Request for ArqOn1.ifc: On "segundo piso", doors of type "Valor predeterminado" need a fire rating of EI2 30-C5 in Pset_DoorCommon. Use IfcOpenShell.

First a look at what the model holds.

```python
import ifcopenshell
import ifcopenshell.util.element

model = ifcopenshell.open("ArqOn1.ifc")
print(model.schema)
storey = next(s for s in model.by_type("IfcBuildingStorey") if s.Name == "segundo piso")
doors = [e for e in ifcopenshell.util.element.get_decomposition(storey) if e.is_a("IfcDoor")]
seen = {}
for e in doors:
    element_type = ifcopenshell.util.element.get_type(e)
    key = (element_type.Name if element_type != e and element_type else None, ifcopenshell.util.element.get_pset(e, "Pset_DoorCommon", "FireRating"))
    seen[key] = seen.get(key, 0) + 1
for (name, value), count in sorted(seen.items(), key=str):
    print(count, "x", name, "|", value)
```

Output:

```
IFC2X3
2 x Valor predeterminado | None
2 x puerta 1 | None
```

```python
import ifcopenshell
import ifcopenshell.api.pset
import ifcopenshell.util.element

model = ifcopenshell.open("ArqOn1.ifc")

storey = next(s for s in model.by_type("IfcBuildingStorey") if s.Name == "segundo piso")
doors = [e for e in ifcopenshell.util.element.get_decomposition(storey) if e.is_a("IfcDoor")]

count = 0
for e in doors:
    element_type = ifcopenshell.util.element.get_type(e)
    if element_type in (None, e) or element_type.Name != "Valor predeterminado":
        continue
    # add_pset returns the element's existing set when there is one.
    pset = ifcopenshell.api.pset.add_pset(model, product=e, name="Pset_DoorCommon")
    ifcopenshell.api.pset.edit_pset(model, pset=pset, properties={"FireRating": "EI2 30-C5"})
    count += 1

print(count, "doors updated")

model.write("ArqOn1_rev.ifc")
```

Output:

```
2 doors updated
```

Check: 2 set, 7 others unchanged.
